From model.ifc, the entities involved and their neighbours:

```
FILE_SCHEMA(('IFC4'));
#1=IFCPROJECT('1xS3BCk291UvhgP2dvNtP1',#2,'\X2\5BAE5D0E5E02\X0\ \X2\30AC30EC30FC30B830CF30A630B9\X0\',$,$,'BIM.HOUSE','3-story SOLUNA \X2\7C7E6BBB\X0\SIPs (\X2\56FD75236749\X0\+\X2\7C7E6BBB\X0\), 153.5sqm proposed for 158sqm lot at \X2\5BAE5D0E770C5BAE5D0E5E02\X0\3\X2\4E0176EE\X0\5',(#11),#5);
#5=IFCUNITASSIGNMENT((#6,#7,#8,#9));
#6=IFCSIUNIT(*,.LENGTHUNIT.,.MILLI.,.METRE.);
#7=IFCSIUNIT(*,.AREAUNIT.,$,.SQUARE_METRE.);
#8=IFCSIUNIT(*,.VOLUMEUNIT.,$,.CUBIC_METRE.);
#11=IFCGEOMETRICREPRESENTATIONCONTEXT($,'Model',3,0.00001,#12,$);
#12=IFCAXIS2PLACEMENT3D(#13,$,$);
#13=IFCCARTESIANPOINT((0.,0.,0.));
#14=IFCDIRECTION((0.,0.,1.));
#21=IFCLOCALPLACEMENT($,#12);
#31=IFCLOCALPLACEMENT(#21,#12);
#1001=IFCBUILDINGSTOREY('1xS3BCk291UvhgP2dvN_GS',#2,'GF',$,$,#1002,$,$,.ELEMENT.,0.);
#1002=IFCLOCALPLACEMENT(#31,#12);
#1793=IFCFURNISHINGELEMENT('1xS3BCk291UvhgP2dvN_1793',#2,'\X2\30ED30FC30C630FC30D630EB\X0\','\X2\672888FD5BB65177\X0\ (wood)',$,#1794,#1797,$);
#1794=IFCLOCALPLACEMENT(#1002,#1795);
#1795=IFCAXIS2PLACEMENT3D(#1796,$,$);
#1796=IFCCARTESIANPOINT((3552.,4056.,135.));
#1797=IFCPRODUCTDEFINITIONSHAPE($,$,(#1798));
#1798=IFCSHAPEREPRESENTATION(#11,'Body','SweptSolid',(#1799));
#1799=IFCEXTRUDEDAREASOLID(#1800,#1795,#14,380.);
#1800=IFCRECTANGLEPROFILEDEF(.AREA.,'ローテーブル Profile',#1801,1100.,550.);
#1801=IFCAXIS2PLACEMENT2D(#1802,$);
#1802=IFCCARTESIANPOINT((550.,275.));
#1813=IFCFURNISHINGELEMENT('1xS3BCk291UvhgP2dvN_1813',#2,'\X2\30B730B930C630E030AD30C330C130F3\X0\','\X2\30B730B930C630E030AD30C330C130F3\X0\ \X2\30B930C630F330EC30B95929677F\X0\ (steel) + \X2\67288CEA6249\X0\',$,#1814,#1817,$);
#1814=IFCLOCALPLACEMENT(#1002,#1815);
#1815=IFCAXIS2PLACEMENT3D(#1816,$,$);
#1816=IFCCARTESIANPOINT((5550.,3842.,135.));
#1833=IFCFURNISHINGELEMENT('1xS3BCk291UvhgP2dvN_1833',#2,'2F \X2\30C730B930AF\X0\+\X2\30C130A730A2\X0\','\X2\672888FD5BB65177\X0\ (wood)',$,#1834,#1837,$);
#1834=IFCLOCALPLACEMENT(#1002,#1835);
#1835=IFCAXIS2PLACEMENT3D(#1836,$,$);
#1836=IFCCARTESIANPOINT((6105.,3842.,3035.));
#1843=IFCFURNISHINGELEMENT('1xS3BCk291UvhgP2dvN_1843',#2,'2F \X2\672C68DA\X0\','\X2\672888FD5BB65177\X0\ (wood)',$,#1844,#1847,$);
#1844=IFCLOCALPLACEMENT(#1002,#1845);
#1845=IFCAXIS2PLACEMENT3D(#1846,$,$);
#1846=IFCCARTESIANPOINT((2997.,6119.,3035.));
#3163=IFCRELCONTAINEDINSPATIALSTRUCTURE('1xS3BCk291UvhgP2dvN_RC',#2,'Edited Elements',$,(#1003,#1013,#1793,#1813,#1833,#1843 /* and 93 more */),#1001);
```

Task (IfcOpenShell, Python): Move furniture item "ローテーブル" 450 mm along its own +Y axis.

```python
import ifcopenshell
import ifcopenshell.api.geometry
import ifcopenshell.util.placement
import ifcopenshell.util.unit

model = ifcopenshell.open("model.ifc")
unit_scale = ifcopenshell.util.unit.calculate_unit_scale(model)

item = model.by_guid("1xS3BCk291UvhgP2dvN_1793")
matrix = ifcopenshell.util.placement.get_local_placement(item.ObjectPlacement)
matrix[:3, 3] += matrix[:3, 1] * 0.45 / unit_scale
ifcopenshell.api.geometry.edit_object_placement(model, product=item, matrix=matrix, is_si=False)

print(ifcopenshell.util.placement.get_local_placement(item.ObjectPlacement).round(3) + 0.0)

model.write("model_updated.ifc")
```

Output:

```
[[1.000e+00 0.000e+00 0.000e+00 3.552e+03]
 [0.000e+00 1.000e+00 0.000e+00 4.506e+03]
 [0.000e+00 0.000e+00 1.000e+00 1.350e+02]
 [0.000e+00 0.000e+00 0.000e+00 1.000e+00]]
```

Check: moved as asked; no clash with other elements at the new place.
